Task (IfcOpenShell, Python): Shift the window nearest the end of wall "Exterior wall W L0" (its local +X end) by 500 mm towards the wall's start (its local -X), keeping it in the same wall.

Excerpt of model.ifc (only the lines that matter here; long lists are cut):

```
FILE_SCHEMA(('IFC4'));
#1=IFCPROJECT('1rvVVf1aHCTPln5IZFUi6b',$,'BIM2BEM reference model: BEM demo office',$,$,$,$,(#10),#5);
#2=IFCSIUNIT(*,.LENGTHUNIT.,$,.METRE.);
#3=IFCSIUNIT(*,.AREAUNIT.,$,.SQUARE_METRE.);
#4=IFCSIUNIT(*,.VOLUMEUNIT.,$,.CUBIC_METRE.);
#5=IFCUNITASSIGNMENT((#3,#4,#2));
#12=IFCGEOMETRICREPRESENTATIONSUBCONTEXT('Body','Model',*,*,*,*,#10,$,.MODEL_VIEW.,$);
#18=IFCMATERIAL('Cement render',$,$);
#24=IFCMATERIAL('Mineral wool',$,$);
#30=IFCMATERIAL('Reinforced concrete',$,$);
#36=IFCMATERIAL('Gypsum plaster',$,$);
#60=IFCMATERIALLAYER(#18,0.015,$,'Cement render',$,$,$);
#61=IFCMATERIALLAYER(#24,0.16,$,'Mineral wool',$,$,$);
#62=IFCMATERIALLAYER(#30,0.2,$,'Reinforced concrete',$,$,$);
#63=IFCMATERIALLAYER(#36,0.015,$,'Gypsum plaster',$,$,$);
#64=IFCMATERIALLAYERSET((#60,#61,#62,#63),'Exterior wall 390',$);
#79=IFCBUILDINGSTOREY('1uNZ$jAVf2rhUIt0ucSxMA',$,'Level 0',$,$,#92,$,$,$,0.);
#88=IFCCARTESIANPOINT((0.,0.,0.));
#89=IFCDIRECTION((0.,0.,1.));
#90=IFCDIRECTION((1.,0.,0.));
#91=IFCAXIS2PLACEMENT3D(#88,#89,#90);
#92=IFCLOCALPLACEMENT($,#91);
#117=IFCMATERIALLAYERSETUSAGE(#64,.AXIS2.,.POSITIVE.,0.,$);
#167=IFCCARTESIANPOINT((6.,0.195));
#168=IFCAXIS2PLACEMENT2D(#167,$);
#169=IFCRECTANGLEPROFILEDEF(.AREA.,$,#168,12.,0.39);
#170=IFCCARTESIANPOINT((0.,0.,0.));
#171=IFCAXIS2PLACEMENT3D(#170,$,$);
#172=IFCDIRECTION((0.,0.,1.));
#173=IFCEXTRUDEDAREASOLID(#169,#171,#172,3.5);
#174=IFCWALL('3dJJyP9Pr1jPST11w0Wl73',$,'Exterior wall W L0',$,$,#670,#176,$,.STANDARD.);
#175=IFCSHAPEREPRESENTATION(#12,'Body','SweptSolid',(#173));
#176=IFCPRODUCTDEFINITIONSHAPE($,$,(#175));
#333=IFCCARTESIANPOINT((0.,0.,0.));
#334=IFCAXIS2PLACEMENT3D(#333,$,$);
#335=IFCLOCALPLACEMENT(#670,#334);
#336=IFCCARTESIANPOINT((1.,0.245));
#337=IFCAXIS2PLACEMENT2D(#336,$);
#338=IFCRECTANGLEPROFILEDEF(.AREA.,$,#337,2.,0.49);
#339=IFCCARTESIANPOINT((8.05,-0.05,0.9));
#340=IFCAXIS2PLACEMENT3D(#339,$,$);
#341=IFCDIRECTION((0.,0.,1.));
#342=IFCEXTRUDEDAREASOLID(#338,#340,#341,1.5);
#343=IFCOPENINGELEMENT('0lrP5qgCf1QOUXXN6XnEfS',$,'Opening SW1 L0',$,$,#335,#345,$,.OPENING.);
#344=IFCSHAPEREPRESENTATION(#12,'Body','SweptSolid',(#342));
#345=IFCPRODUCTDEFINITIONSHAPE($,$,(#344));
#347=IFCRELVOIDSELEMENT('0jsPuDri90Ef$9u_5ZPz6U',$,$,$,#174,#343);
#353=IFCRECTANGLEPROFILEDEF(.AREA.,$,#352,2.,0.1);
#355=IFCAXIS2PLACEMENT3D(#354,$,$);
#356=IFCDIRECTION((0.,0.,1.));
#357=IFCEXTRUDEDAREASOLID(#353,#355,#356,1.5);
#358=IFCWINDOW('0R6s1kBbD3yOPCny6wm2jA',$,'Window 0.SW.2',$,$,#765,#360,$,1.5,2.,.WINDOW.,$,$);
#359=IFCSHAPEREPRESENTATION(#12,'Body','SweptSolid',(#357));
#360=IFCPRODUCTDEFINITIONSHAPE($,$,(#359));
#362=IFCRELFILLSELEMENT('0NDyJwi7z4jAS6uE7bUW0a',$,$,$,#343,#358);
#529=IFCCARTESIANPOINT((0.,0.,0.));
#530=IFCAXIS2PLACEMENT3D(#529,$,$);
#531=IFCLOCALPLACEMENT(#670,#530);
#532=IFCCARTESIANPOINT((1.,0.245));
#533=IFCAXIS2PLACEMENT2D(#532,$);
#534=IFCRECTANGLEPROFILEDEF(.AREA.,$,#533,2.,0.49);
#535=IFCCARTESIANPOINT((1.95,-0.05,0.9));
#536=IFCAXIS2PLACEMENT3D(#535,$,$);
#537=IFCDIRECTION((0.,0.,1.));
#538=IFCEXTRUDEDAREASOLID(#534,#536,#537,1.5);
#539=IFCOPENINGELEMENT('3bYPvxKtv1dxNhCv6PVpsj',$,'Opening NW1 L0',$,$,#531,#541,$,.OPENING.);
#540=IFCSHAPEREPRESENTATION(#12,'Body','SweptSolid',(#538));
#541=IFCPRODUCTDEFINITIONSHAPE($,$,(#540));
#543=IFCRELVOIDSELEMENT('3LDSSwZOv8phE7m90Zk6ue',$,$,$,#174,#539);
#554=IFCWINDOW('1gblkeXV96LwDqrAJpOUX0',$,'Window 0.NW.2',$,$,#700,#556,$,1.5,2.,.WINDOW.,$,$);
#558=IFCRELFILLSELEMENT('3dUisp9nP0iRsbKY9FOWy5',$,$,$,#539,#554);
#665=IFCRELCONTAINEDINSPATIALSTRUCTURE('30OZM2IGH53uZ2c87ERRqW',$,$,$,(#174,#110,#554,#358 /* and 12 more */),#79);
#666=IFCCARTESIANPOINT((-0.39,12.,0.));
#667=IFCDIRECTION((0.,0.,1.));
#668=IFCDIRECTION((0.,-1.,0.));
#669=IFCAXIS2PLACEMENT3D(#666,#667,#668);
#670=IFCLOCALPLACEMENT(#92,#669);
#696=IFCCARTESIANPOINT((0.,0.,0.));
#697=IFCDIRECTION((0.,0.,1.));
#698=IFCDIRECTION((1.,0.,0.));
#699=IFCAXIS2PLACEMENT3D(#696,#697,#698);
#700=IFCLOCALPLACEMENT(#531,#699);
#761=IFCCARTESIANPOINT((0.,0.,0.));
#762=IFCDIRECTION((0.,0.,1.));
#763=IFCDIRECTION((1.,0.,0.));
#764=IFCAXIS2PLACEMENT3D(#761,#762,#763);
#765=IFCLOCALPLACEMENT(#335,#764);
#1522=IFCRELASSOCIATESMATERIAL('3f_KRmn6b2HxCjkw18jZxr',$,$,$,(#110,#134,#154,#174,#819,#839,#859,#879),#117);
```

```python
import ifcopenshell
import ifcopenshell.api.geometry
import ifcopenshell.util.placement
import ifcopenshell.util.unit

model = ifcopenshell.open("model.ifc")
unit_scale = ifcopenshell.util.unit.calculate_unit_scale(model)

window = model.by_guid("0R6s1kBbD3yOPCny6wm2jA")
opening = window.FillsVoids[0].RelatingOpeningElement
wall = opening.VoidsElements[0].RelatingBuildingElement

wall_matrix = ifcopenshell.util.placement.get_local_placement(wall.ObjectPlacement)
shift = wall_matrix[:3, 0] * -0.5 / unit_scale
before = ifcopenshell.util.placement.get_local_placement(window.ObjectPlacement)[:3, 3].copy()

# The window is placed relative to its opening, so it follows when the opening moves.
matrix = ifcopenshell.util.placement.get_local_placement(opening.ObjectPlacement)
matrix[:3, 3] += shift
ifcopenshell.api.geometry.edit_object_placement(
    model, product=opening, matrix=matrix, is_si=False, should_transform_children=True
)

after = ifcopenshell.util.placement.get_local_placement(window.ObjectPlacement)[:3, 3]
print("window moved by", (after - before).round(3) + 0.0)

model.write("model_edited.ifc")
```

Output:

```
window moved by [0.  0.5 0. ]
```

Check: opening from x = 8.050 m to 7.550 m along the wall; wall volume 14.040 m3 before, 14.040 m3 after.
